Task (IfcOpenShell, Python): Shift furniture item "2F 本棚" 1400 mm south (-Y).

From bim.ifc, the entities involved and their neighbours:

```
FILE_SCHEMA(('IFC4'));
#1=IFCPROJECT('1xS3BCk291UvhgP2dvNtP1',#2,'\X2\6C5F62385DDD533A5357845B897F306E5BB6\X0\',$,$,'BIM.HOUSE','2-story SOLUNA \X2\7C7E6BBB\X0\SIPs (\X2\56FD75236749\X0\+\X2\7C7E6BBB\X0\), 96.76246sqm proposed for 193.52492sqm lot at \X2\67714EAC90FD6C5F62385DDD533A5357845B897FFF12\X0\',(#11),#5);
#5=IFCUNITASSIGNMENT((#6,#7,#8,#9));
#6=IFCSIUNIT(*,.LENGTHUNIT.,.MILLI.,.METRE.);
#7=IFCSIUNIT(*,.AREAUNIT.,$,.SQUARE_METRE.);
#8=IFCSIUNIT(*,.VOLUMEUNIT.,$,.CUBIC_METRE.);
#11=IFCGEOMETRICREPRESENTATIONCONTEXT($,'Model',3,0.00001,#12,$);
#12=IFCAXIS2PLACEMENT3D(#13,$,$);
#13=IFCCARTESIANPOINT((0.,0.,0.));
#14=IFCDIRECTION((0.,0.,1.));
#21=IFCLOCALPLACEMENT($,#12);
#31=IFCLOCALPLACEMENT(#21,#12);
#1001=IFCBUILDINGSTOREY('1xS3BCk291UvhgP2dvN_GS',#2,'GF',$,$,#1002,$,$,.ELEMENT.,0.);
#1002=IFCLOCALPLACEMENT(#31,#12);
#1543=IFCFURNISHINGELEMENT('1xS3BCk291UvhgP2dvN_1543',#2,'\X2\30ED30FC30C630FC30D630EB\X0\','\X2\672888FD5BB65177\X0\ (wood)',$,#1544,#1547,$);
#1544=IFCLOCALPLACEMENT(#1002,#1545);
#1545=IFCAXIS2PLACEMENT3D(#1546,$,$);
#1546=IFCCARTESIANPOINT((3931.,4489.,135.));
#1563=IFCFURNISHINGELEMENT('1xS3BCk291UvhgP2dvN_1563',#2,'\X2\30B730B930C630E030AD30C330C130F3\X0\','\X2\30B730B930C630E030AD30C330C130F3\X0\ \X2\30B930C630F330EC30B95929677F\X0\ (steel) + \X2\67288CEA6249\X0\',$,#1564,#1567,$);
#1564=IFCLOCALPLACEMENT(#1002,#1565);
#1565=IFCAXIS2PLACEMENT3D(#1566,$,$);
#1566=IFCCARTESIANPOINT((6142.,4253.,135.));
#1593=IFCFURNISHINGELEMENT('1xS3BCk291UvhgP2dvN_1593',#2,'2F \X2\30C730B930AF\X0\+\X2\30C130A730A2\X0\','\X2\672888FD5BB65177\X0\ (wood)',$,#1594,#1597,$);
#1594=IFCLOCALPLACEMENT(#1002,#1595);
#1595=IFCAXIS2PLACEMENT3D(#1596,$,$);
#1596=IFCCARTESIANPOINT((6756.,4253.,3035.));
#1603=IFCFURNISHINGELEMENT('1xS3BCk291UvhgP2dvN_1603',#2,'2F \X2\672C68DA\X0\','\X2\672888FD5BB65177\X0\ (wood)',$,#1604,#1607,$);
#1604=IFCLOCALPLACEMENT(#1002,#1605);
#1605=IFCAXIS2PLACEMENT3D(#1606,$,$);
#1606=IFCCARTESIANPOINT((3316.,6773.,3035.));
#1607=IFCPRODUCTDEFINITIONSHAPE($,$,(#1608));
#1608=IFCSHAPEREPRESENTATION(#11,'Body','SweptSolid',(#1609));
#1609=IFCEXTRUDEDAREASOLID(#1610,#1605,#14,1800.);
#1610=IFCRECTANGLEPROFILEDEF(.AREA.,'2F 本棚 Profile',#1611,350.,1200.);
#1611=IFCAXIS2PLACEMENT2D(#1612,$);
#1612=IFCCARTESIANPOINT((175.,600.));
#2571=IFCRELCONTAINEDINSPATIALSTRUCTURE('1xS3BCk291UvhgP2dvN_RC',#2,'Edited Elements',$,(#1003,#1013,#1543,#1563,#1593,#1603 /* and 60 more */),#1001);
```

```python
import ifcopenshell
import ifcopenshell.api.geometry
import ifcopenshell.util.placement

model = ifcopenshell.open("bim.ifc")

item = model.by_guid("1xS3BCk291UvhgP2dvN_1603")
matrix = ifcopenshell.util.placement.get_local_placement(item.ObjectPlacement)
matrix[1, 3] -= 1400.0
ifcopenshell.api.geometry.edit_object_placement(model, product=item, matrix=matrix, is_si=False)

print(ifcopenshell.util.placement.get_local_placement(item.ObjectPlacement).round(3) + 0.0)

model.write("bim-out.ifc")
```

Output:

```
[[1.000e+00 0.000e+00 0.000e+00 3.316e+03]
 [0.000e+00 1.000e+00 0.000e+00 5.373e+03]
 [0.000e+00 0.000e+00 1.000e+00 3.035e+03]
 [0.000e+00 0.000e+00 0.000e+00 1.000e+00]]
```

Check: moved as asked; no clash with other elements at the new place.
